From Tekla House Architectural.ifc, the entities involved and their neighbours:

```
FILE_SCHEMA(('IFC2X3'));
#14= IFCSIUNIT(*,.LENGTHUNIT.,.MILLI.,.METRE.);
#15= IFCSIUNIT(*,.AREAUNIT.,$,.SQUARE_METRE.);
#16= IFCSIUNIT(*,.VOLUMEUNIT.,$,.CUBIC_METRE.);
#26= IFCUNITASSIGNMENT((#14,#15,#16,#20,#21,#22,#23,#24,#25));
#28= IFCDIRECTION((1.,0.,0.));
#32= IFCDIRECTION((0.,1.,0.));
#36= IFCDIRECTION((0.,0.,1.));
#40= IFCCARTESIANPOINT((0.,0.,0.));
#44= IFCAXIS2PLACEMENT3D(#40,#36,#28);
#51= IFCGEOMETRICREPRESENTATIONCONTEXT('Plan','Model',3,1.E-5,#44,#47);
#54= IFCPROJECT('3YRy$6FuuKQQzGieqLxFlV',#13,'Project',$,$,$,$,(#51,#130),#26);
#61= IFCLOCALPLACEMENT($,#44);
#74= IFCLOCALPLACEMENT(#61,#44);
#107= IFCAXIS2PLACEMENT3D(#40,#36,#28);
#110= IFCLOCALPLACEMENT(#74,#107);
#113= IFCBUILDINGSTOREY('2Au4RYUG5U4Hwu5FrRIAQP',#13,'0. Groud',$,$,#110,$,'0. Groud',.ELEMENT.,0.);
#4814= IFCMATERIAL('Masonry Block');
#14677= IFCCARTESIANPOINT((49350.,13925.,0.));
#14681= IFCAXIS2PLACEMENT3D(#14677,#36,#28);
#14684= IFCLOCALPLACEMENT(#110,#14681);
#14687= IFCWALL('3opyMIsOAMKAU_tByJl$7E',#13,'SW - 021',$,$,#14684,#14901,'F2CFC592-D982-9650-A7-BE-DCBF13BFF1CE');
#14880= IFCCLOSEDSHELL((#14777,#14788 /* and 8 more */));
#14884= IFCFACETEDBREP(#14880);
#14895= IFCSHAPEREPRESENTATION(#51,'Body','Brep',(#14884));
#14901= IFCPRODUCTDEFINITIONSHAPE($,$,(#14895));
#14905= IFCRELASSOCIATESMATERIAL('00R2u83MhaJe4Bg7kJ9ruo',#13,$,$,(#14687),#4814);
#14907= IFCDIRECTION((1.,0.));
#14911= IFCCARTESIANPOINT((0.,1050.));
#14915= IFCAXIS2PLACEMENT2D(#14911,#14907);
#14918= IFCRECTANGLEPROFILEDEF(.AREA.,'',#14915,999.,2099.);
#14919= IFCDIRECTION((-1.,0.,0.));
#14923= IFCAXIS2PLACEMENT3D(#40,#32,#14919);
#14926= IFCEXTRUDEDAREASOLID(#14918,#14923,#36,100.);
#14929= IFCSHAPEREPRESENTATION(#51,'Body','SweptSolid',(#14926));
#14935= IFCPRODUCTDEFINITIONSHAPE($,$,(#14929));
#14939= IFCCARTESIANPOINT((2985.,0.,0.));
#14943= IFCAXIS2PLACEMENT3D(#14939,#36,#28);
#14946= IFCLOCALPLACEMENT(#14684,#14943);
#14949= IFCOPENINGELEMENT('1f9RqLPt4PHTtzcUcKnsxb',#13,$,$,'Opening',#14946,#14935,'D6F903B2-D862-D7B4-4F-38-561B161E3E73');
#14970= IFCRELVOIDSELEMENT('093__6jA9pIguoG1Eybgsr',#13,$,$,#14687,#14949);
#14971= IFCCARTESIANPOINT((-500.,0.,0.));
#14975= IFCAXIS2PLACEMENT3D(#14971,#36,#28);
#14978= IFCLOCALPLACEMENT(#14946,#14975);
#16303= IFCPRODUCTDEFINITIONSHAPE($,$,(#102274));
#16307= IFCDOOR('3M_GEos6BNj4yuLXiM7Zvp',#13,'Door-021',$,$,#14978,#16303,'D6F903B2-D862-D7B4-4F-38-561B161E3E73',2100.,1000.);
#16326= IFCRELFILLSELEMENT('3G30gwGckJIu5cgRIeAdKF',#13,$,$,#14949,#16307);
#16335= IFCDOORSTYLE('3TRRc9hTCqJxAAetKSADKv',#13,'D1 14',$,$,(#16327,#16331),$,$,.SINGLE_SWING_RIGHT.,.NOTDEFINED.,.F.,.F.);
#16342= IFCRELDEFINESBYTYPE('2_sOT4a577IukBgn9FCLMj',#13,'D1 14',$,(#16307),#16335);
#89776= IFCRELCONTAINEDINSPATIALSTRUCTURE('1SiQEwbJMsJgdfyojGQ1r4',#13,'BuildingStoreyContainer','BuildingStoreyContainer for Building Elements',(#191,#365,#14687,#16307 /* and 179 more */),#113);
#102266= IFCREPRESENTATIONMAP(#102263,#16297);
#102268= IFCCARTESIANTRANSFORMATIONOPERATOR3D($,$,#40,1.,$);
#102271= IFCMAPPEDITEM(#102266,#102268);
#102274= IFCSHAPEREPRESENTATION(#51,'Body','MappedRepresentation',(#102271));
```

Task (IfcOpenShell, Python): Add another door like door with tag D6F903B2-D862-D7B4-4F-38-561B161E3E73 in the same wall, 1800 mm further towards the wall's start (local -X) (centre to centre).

```python
import ifcopenshell
import ifcopenshell.api.feature
import ifcopenshell.api.geometry
import ifcopenshell.api.root
import ifcopenshell.geom
import ifcopenshell.util.element
import ifcopenshell.util.placement
import ifcopenshell.util.shape

model = ifcopenshell.open("Tekla House Architectural.ifc")
settings = ifcopenshell.geom.settings()


def volume(element):
    """Net volume in cubic metres, openings subtracted."""
    shape = ifcopenshell.geom.create_shape(settings, element)
    return ifcopenshell.util.shape.get_volume(shape.geometry)


door = model.by_guid("3M_GEos6BNj4yuLXiM7Zvp")
opening = door.FillsVoids[0].RelatingOpeningElement
wall = opening.VoidsElements[0].RelatingBuildingElement
before = volume(wall)
shift = ifcopenshell.util.placement.get_local_placement(wall.ObjectPlacement)[:3, 0] * -1800.0

# copy_class copies the void relationship, type, container and properties, but no geometry.
new_opening = ifcopenshell.api.root.copy_class(model, product=opening)
new_opening.Representation = ifcopenshell.util.element.copy_deep(
    model, opening.Representation, exclude=["IfcGeometricRepresentationContext", "IfcRepresentationMap"]
)
new_opening.Tag = None
new_door = ifcopenshell.api.root.copy_class(model, product=door)
new_door.Representation = ifcopenshell.util.element.copy_deep(
    model, door.Representation, exclude=["IfcGeometricRepresentationContext", "IfcRepresentationMap"]
)
new_door.Tag = None
fills = ifcopenshell.api.feature.add_filling(model, opening=new_opening, element=new_door)
fills.OwnerHistory = new_door.OwnerHistory  # required in IFC2X3

for old, new in ((opening, new_opening), (door, new_door)):
    matrix = ifcopenshell.util.placement.get_local_placement(old.ObjectPlacement)
    matrix[:3, 3] += shift
    ifcopenshell.api.geometry.edit_object_placement(model, product=new, matrix=matrix, is_si=False)

after = volume(wall)

print(f"wall volume {before:.3f} -> {after:.3f} m3")

model.write("Tekla House Architectural_edited.ifc")
```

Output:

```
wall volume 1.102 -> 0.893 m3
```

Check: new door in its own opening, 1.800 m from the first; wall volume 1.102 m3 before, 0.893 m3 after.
